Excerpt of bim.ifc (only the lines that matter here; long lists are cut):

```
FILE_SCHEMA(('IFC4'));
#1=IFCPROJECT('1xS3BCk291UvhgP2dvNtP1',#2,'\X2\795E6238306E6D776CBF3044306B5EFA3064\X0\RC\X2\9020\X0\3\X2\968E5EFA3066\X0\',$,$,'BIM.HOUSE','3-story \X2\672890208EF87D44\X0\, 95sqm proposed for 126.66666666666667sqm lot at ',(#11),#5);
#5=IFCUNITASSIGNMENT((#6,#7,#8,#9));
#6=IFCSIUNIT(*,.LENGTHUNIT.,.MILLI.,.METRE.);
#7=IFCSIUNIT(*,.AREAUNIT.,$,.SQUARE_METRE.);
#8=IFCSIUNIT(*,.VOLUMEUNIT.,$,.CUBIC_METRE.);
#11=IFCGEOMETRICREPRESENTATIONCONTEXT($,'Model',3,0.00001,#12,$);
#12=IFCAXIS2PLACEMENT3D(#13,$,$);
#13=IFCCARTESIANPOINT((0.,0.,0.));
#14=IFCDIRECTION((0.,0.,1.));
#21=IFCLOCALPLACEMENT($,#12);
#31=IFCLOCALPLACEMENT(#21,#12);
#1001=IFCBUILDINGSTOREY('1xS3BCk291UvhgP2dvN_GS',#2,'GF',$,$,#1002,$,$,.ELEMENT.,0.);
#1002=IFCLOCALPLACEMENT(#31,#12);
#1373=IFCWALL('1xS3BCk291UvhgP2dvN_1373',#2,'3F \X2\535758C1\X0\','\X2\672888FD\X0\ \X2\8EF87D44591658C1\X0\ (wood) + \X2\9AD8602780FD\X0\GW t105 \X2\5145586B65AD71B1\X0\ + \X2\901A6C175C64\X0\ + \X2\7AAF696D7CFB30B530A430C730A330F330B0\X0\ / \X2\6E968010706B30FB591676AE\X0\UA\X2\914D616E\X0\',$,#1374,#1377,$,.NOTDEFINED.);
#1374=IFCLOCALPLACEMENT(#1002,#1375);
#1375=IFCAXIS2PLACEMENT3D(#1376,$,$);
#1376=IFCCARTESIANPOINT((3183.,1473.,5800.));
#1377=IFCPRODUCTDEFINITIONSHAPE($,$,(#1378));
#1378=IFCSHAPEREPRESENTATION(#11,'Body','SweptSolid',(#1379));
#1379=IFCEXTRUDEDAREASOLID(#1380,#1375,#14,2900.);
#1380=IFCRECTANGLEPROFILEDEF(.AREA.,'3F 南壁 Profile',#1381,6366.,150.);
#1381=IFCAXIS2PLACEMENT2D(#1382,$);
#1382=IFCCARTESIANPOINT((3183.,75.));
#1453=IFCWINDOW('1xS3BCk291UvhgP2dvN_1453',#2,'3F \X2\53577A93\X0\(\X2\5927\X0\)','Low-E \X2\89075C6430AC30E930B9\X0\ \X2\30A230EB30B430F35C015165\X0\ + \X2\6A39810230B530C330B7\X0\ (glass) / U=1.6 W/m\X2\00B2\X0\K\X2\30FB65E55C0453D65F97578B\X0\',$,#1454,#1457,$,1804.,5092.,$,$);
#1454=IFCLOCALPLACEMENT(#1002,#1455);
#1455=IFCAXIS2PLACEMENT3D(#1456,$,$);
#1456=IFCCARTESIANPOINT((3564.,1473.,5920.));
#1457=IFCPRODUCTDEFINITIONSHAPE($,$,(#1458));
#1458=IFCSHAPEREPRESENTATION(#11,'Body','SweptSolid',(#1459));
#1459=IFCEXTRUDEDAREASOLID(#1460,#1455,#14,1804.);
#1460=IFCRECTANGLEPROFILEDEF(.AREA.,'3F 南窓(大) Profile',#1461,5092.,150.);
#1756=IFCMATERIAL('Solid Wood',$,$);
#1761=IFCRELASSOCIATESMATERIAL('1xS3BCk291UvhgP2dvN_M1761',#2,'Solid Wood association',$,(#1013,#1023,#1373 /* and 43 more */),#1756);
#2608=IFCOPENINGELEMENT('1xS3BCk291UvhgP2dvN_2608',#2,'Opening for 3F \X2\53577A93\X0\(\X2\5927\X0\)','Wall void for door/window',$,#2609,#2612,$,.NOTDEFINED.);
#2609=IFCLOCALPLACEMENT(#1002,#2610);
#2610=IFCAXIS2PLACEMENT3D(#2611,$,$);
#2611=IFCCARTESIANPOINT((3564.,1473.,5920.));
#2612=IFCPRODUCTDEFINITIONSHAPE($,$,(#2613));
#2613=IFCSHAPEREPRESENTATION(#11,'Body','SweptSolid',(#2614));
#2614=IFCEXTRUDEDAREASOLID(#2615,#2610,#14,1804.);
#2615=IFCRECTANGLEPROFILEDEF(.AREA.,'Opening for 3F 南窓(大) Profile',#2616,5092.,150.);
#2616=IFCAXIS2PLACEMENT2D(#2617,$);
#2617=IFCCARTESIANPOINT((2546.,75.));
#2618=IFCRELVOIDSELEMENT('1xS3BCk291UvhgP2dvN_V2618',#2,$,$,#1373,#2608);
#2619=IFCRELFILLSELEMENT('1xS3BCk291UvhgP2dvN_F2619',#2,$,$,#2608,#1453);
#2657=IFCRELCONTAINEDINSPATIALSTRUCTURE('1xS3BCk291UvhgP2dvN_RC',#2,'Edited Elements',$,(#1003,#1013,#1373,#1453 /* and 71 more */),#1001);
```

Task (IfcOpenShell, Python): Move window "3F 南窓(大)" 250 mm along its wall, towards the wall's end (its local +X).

```python
import ifcopenshell
import ifcopenshell.api.geometry
import ifcopenshell.util.placement

model = ifcopenshell.open("bim.ifc")

window = model.by_guid("1xS3BCk291UvhgP2dvN_1453")
opening = window.FillsVoids[0].RelatingOpeningElement
wall = opening.VoidsElements[0].RelatingBuildingElement

wall_matrix = ifcopenshell.util.placement.get_local_placement(wall.ObjectPlacement)
shift = wall_matrix[:3, 0] * 250.0
before = ifcopenshell.util.placement.get_local_placement(window.ObjectPlacement)[:3, 3].copy()

# The window is not placed relative to its opening, so move both.
for product in (opening, window):
    matrix = ifcopenshell.util.placement.get_local_placement(product.ObjectPlacement)
    matrix[:3, 3] += shift
    ifcopenshell.api.geometry.edit_object_placement(model, product=product, matrix=matrix, is_si=False)

after = ifcopenshell.util.placement.get_local_placement(window.ObjectPlacement)[:3, 3]
print("window moved by", (after - before).round(3) + 0.0)

model.write("bim_updated.ifc")
```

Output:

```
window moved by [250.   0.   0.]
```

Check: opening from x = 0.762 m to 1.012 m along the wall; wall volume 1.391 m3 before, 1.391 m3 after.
